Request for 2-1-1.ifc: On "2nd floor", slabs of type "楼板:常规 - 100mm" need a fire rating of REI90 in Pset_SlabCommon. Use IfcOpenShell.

First a look at what the model holds.

```python
import ifcopenshell
import ifcopenshell.util.element

model = ifcopenshell.open("2-1-1.ifc")
print(model.schema)
storey = next(s for s in model.by_type("IfcBuildingStorey") if s.Name == "2nd floor")
slabs = [e for e in ifcopenshell.util.element.get_decomposition(storey) if e.is_a("IfcSlab")]
seen = {}
for e in slabs:
    element_type = ifcopenshell.util.element.get_type(e)
    key = (element_type.Name if element_type != e and element_type else None, ifcopenshell.util.element.get_pset(e, "Pset_SlabCommon", "FireRating"))
    seen[key] = seen.get(key, 0) + 1
for (name, value), count in sorted(seen.items(), key=str):
    print(count, "x", name, "|", value)
```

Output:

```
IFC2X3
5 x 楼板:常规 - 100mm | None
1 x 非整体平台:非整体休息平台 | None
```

```python
import ifcopenshell
import ifcopenshell.api.pset
import ifcopenshell.util.element

model = ifcopenshell.open("2-1-1.ifc")

storey = next(s for s in model.by_type("IfcBuildingStorey") if s.Name == "2nd floor")
slabs = [e for e in ifcopenshell.util.element.get_decomposition(storey) if e.is_a("IfcSlab")]

count = 0
for e in slabs:
    element_type = ifcopenshell.util.element.get_type(e)
    if element_type in (None, e) or element_type.Name != "楼板:常规 - 100mm":
        continue
    # add_pset returns the element's existing set when there is one.
    pset = ifcopenshell.api.pset.add_pset(model, product=e, name="Pset_SlabCommon")
    ifcopenshell.api.pset.edit_pset(model, pset=pset, properties={"FireRating": "REI90"})
    count += 1

print(count, "slabs updated")

model.write("2-1-1-out.ifc")
```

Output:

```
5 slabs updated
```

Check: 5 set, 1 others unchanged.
